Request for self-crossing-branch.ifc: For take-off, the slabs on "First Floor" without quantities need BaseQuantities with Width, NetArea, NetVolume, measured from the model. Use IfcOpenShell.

First a look at what the model holds.

```python
import ifcopenshell
import ifcopenshell.util.element
import ifcopenshell.util.unit

model = ifcopenshell.open("self-crossing-branch.ifc")
print(model.schema)
for unit_type in ("LENGTHUNIT", "AREAUNIT", "VOLUMEUNIT"):
    print(unit_type, ifcopenshell.util.unit.calculate_unit_scale(model, unit_type))
storey = next(s for s in model.by_type("IfcBuildingStorey") if s.Name == "First Floor")
slabs = [e for e in ifcopenshell.util.element.get_decomposition(storey) if e.is_a("IfcSlab")]
for e in sorted(slabs, key=lambda e: e.id()):
    print(e.id(), e.is_a(), e.Name, list(ifcopenshell.util.element.get_psets(e, qtos_only=True)), sep=" | ")
```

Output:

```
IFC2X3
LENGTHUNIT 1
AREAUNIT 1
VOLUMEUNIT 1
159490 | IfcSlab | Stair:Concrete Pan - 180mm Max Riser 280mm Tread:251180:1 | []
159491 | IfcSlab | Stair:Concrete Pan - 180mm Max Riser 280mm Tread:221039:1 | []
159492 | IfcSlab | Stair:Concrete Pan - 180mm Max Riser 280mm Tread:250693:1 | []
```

```python
import ifcopenshell
import ifcopenshell.api.pset
import ifcopenshell.geom
import ifcopenshell.util.element
import ifcopenshell.util.shape
import ifcopenshell.util.unit

model = ifcopenshell.open("self-crossing-branch.ifc")
unit_scale = ifcopenshell.util.unit.calculate_unit_scale(model)
area_scale = ifcopenshell.util.unit.calculate_unit_scale(model, "AREAUNIT")
volume_scale = ifcopenshell.util.unit.calculate_unit_scale(model, "VOLUMEUNIT")
settings = ifcopenshell.geom.settings()

storey = next(s for s in model.by_type("IfcBuildingStorey") if s.Name == "First Floor")
slabs = [e for e in ifcopenshell.util.element.get_decomposition(storey) if e.is_a("IfcSlab")]

for e in sorted(slabs, key=lambda e: e.id()):
    if ifcopenshell.util.element.get_psets(e, qtos_only=True, should_inherit=False):
        continue
    # Geometry comes back in metres, in the element's own axes.
    shape = ifcopenshell.geom.create_shape(settings, e)
    values = {
        "Width": ifcopenshell.util.shape.get_z(shape.geometry) / unit_scale,
        "NetArea": ifcopenshell.util.shape.get_footprint_area(shape.geometry) / area_scale,
        "NetVolume": ifcopenshell.util.shape.get_volume(shape.geometry) / volume_scale,
    }
    qto = ifcopenshell.api.pset.add_qto(model, product=e, name="BaseQuantities")
    ifcopenshell.api.pset.edit_qto(model, qto=qto, properties=values)
    print(e.id(), {k: round(v, 3) for k, v in values.items()})

model.write("self-crossing-branch_rev.ifc")
```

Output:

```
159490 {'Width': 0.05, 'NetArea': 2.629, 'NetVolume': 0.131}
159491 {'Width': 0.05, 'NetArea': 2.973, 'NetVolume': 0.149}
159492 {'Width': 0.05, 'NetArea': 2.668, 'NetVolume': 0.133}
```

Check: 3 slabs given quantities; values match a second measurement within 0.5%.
